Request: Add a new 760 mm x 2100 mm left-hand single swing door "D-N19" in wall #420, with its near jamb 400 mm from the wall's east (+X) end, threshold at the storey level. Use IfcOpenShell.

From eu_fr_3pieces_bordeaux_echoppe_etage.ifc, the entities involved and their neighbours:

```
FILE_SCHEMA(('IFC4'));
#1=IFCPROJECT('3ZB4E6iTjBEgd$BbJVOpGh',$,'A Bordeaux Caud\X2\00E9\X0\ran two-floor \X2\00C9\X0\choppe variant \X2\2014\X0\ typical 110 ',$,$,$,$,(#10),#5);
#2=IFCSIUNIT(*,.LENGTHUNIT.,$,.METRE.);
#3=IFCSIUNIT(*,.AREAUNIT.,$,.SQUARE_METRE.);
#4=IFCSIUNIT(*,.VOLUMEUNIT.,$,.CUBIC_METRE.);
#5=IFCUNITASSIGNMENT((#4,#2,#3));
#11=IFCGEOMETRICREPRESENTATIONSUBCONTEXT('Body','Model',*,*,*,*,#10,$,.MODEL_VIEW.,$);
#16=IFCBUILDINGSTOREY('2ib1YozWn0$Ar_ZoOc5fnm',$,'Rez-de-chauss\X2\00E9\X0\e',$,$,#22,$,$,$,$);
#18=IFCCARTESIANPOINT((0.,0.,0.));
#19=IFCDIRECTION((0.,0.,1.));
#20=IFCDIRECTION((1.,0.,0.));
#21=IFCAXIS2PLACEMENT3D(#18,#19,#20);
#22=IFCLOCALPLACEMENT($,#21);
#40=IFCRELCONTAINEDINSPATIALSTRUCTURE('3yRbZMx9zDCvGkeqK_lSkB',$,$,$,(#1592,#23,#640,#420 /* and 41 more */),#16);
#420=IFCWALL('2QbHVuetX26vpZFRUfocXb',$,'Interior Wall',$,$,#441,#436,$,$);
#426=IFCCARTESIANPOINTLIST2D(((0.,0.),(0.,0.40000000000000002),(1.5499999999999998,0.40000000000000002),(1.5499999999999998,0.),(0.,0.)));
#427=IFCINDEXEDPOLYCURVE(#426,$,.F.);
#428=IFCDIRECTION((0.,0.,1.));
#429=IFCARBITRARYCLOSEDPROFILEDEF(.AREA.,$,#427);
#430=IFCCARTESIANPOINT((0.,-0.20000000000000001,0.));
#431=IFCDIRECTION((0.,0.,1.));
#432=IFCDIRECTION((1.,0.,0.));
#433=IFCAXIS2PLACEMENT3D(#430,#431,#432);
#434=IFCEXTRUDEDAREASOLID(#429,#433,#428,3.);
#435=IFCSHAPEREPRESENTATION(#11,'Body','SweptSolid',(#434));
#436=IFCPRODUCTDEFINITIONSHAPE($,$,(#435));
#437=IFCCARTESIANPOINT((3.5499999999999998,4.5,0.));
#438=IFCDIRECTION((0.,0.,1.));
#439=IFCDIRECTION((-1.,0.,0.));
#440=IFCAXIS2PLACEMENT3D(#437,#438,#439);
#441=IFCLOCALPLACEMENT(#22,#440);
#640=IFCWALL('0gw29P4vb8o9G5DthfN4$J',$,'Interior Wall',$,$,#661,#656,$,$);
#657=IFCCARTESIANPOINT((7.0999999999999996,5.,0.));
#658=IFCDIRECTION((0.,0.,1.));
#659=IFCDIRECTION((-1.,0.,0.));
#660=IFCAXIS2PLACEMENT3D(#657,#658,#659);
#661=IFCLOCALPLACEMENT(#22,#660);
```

```python
import numpy as np
import ifcopenshell
import ifcopenshell.api.feature
import ifcopenshell.api.geometry
import ifcopenshell.api.root
import ifcopenshell.api.spatial
import ifcopenshell.geom
import ifcopenshell.util.element
import ifcopenshell.util.placement
import ifcopenshell.util.representation
import ifcopenshell.util.shape
import ifcopenshell.util.unit

model = ifcopenshell.open("eu_fr_3pieces_bordeaux_echoppe_etage.ifc")
unit_scale = ifcopenshell.util.unit.calculate_unit_scale(model)
settings = ifcopenshell.geom.settings()


def volume(element):
    """Net volume in cubic metres, openings subtracted."""
    shape = ifcopenshell.geom.create_shape(settings, element)
    return ifcopenshell.util.shape.get_volume(shape.geometry)


wall = model.by_id(420)
storey = ifcopenshell.util.element.get_container(wall, ifc_class="IfcBuildingStorey")
context = ifcopenshell.util.representation.get_context(model, "Model", "Body", "MODEL_VIEW")
before = volume(wall)

width, height, from_end, sill = 0.76, 2.1, 0.4, 0.0  # metres

# The wall runs along its own X axis, and the end named is its -X end.
wall_shape = ifcopenshell.geom.create_shape(settings, wall)
x, y, z = ifcopenshell.util.shape.get_vertices(wall_shape.geometry).T
start = x.min() + from_end
face, thickness = float(y.min()), float(y.max() - y.min())
wall_matrix = ifcopenshell.util.placement.get_local_placement(wall.ObjectPlacement)
level = ifcopenshell.util.placement.get_local_placement(storey.ObjectPlacement)[2, 3]


def in_wall(x, y):
    """Placement at x, y metres in the wall's axes, at sill height."""
    matrix = wall_matrix.copy()
    matrix[:, 3] = wall_matrix @ np.array([x / unit_scale, y / unit_scale, 0.0, 1.0])
    matrix[2, 3] = level + sill / unit_scale
    return matrix


# Opening: a box that overshoots both wall faces by 50 mm.
opening = ifcopenshell.api.root.create_entity(model, ifc_class="IfcOpeningElement", predefined_type="OPENING")
box = ifcopenshell.api.geometry.add_wall_representation(
    model, context=context, length=width, height=height, thickness=thickness + 0.1
)
ifcopenshell.api.geometry.assign_representation(model, product=opening, representation=box)
ifcopenshell.api.geometry.edit_object_placement(model, product=opening, matrix=in_wall(start, face - 0.05), is_si=False)
ifcopenshell.api.feature.add_feature(model, feature=opening, element=wall)

door = ifcopenshell.api.root.create_entity(model, ifc_class="IfcDoor", name="D-N19", predefined_type="DOOR")
door.OverallWidth, door.OverallHeight = width / unit_scale, height / unit_scale
door.OperationType = "SINGLE_SWING_LEFT"
body = ifcopenshell.api.geometry.add_door_representation(
    model,
    context=context,
    overall_width=door.OverallWidth,
    overall_height=door.OverallHeight,
    operation_type="SINGLE_SWING_LEFT",
    lining_properties={"LiningDepth": thickness / unit_scale, "ThresholdDepth": thickness / unit_scale},
)
ifcopenshell.api.geometry.assign_representation(model, product=door, representation=body)
ifcopenshell.api.spatial.assign_container(model, products=[door], relating_structure=storey)
ifcopenshell.api.feature.add_filling(model, opening=opening, element=door)

# The lining spans the wall, so the door starts at the wall face.
ifcopenshell.api.geometry.edit_object_placement(model, product=door, matrix=in_wall(start, face), is_si=False)

after = volume(wall)

print(f"wall volume {before:.3f} -> {after:.3f} m3")

model.write("eu_fr_3pieces_bordeaux_echoppe_etage_updated.ifc")
```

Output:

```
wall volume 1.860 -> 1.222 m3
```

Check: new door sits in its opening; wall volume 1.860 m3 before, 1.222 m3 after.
